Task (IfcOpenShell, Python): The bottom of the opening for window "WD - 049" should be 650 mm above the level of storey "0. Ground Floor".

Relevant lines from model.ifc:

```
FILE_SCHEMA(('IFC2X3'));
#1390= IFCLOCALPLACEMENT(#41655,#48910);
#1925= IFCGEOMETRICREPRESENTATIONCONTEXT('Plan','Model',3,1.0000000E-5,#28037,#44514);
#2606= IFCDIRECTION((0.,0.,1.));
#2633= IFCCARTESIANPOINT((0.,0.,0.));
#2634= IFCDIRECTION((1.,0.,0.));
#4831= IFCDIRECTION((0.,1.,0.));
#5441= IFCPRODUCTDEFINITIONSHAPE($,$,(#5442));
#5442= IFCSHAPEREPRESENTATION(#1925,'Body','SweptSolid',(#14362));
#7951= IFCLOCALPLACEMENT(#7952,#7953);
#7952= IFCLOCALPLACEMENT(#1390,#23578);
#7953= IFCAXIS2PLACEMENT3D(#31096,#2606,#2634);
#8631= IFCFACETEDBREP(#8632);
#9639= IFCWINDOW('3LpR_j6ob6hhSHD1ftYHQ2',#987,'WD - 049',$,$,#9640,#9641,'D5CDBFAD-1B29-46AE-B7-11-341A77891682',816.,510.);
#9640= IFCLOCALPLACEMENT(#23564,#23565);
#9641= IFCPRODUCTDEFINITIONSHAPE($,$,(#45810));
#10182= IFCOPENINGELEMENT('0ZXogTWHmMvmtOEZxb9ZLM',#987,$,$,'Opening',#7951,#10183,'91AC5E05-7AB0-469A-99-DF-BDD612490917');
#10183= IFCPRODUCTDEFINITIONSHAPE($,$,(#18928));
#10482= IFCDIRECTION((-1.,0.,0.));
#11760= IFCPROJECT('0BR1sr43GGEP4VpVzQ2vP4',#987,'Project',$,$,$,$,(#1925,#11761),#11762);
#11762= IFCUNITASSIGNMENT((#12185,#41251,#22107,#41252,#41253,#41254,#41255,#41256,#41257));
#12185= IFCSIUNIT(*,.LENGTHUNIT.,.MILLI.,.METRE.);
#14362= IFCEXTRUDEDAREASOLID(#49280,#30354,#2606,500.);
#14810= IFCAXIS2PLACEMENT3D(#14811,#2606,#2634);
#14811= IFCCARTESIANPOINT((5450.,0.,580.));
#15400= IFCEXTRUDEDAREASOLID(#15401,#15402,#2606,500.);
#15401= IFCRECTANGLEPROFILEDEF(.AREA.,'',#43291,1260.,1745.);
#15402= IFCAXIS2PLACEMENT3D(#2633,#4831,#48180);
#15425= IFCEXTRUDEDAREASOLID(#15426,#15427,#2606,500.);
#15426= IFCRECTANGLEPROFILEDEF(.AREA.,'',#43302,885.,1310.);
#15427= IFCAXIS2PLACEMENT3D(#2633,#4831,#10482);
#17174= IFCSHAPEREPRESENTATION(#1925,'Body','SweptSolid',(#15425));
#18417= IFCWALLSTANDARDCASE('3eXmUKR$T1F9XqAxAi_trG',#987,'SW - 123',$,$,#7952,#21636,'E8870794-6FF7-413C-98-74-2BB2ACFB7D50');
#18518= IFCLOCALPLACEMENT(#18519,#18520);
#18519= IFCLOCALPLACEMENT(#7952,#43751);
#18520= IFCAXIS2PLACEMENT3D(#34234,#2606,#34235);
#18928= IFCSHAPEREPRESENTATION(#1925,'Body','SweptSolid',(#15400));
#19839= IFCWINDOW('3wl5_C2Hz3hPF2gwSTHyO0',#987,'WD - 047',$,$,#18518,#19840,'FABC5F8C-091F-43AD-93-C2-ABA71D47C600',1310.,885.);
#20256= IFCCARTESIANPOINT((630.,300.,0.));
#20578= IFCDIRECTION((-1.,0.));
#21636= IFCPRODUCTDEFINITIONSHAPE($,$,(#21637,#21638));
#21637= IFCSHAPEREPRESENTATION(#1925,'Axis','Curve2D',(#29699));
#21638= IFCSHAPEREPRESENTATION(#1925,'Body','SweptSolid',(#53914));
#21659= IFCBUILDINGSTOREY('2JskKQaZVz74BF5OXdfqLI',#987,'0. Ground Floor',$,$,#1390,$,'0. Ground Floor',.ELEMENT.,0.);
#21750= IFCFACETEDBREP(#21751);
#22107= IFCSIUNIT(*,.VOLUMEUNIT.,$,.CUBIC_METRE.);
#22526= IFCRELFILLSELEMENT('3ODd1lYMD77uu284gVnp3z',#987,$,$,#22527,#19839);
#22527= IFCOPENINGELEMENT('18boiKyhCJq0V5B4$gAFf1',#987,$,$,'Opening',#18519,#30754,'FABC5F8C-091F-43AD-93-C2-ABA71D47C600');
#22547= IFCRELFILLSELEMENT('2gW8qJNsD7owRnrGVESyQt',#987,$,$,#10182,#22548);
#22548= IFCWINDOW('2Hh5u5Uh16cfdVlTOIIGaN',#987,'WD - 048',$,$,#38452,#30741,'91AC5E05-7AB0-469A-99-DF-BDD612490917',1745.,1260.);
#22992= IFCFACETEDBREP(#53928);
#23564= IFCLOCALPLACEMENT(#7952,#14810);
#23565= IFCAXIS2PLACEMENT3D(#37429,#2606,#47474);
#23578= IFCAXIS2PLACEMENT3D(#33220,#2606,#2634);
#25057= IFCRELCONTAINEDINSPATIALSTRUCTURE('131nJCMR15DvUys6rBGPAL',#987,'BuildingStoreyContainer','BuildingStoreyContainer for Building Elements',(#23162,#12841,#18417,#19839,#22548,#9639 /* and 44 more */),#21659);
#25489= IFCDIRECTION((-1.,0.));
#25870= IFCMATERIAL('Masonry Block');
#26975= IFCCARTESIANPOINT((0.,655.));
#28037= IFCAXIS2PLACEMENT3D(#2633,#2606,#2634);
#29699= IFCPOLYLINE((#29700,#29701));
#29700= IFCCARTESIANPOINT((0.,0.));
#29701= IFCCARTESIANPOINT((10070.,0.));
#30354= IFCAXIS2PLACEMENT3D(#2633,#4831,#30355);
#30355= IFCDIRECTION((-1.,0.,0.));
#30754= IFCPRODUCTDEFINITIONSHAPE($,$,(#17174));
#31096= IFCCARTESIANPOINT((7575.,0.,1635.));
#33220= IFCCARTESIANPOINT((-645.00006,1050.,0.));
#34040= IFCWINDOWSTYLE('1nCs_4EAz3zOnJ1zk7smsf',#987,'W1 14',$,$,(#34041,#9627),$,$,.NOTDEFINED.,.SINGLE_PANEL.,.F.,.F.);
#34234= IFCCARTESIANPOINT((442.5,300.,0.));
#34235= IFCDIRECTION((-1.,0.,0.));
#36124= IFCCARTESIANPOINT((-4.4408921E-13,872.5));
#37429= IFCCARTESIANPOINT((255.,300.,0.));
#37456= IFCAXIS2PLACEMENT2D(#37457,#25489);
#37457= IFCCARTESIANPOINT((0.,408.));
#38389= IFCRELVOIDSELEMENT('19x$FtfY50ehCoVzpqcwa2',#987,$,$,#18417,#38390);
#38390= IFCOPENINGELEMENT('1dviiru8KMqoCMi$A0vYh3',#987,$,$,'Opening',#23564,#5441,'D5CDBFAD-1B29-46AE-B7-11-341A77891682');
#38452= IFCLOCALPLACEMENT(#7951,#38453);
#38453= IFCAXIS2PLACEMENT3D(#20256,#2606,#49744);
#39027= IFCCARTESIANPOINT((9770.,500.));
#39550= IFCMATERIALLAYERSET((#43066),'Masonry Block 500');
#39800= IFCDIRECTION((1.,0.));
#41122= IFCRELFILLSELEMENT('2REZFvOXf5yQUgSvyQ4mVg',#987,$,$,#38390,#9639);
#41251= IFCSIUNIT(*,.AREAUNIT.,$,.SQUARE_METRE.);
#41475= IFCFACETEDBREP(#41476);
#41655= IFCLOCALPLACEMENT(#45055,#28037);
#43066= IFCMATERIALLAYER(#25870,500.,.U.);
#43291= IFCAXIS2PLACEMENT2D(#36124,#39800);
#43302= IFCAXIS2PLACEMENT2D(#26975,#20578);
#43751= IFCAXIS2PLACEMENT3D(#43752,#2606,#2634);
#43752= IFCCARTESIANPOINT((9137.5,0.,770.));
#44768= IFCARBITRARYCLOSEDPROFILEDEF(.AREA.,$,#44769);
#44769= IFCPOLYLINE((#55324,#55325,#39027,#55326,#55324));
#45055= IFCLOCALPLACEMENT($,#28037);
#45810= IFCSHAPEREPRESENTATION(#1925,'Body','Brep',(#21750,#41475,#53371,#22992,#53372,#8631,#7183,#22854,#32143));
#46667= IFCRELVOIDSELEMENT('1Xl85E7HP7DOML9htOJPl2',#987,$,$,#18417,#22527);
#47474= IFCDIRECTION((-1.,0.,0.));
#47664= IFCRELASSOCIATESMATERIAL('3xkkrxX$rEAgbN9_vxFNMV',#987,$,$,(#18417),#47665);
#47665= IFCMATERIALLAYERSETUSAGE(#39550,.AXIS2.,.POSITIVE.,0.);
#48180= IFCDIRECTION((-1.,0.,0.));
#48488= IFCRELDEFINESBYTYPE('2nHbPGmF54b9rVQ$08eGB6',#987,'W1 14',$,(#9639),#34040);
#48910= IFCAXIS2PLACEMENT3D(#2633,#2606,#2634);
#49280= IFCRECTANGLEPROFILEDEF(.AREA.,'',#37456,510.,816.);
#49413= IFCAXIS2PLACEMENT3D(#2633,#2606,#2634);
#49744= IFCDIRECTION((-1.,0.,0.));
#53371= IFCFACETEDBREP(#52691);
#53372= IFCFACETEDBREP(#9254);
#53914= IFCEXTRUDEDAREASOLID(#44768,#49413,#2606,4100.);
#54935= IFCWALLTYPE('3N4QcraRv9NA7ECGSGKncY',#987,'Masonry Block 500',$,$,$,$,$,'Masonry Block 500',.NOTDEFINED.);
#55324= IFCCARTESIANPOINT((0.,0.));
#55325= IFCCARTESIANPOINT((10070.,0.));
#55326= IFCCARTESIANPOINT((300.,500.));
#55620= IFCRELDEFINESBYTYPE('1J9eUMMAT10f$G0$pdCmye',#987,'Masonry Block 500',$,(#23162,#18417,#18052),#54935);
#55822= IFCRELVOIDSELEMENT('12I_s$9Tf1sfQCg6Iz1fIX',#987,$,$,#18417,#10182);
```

```python
import numpy as np
import ifcopenshell
import ifcopenshell.api.geometry
import ifcopenshell.geom
import ifcopenshell.util.element
import ifcopenshell.util.placement
import ifcopenshell.util.shape
import ifcopenshell.util.unit

model = ifcopenshell.open("model.ifc")
unit_scale = ifcopenshell.util.unit.calculate_unit_scale(model)

window = model.by_guid("3LpR_j6ob6hhSHD1ftYHQ2")
opening = window.FillsVoids[0].RelatingOpeningElement
storey = ifcopenshell.util.element.get_container(window, ifc_class="IfcBuildingStorey")
level = ifcopenshell.util.placement.get_local_placement(storey.ObjectPlacement)[2, 3]

# The opening's origin need not be at the sill, so measure its lowest point.
shape = ifcopenshell.geom.create_shape(ifcopenshell.geom.settings(), opening)
bottom = ifcopenshell.util.shape.get_shape_bottom_elevation(shape, shape.geometry) / unit_scale
dz = level + 0.65 / unit_scale - bottom

shift = np.array([0.0, 0.0, dz])
# The window is placed relative to its opening, so it follows when the opening moves.
matrix = ifcopenshell.util.placement.get_local_placement(opening.ObjectPlacement)
matrix[:3, 3] += shift
ifcopenshell.api.geometry.edit_object_placement(
    model, product=opening, matrix=matrix, is_si=False, should_transform_children=True
)

print(f"moved by {dz * unit_scale:+.3f} m")

model.write("model-out.ifc")
```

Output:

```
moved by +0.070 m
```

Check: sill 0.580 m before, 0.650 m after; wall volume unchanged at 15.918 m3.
